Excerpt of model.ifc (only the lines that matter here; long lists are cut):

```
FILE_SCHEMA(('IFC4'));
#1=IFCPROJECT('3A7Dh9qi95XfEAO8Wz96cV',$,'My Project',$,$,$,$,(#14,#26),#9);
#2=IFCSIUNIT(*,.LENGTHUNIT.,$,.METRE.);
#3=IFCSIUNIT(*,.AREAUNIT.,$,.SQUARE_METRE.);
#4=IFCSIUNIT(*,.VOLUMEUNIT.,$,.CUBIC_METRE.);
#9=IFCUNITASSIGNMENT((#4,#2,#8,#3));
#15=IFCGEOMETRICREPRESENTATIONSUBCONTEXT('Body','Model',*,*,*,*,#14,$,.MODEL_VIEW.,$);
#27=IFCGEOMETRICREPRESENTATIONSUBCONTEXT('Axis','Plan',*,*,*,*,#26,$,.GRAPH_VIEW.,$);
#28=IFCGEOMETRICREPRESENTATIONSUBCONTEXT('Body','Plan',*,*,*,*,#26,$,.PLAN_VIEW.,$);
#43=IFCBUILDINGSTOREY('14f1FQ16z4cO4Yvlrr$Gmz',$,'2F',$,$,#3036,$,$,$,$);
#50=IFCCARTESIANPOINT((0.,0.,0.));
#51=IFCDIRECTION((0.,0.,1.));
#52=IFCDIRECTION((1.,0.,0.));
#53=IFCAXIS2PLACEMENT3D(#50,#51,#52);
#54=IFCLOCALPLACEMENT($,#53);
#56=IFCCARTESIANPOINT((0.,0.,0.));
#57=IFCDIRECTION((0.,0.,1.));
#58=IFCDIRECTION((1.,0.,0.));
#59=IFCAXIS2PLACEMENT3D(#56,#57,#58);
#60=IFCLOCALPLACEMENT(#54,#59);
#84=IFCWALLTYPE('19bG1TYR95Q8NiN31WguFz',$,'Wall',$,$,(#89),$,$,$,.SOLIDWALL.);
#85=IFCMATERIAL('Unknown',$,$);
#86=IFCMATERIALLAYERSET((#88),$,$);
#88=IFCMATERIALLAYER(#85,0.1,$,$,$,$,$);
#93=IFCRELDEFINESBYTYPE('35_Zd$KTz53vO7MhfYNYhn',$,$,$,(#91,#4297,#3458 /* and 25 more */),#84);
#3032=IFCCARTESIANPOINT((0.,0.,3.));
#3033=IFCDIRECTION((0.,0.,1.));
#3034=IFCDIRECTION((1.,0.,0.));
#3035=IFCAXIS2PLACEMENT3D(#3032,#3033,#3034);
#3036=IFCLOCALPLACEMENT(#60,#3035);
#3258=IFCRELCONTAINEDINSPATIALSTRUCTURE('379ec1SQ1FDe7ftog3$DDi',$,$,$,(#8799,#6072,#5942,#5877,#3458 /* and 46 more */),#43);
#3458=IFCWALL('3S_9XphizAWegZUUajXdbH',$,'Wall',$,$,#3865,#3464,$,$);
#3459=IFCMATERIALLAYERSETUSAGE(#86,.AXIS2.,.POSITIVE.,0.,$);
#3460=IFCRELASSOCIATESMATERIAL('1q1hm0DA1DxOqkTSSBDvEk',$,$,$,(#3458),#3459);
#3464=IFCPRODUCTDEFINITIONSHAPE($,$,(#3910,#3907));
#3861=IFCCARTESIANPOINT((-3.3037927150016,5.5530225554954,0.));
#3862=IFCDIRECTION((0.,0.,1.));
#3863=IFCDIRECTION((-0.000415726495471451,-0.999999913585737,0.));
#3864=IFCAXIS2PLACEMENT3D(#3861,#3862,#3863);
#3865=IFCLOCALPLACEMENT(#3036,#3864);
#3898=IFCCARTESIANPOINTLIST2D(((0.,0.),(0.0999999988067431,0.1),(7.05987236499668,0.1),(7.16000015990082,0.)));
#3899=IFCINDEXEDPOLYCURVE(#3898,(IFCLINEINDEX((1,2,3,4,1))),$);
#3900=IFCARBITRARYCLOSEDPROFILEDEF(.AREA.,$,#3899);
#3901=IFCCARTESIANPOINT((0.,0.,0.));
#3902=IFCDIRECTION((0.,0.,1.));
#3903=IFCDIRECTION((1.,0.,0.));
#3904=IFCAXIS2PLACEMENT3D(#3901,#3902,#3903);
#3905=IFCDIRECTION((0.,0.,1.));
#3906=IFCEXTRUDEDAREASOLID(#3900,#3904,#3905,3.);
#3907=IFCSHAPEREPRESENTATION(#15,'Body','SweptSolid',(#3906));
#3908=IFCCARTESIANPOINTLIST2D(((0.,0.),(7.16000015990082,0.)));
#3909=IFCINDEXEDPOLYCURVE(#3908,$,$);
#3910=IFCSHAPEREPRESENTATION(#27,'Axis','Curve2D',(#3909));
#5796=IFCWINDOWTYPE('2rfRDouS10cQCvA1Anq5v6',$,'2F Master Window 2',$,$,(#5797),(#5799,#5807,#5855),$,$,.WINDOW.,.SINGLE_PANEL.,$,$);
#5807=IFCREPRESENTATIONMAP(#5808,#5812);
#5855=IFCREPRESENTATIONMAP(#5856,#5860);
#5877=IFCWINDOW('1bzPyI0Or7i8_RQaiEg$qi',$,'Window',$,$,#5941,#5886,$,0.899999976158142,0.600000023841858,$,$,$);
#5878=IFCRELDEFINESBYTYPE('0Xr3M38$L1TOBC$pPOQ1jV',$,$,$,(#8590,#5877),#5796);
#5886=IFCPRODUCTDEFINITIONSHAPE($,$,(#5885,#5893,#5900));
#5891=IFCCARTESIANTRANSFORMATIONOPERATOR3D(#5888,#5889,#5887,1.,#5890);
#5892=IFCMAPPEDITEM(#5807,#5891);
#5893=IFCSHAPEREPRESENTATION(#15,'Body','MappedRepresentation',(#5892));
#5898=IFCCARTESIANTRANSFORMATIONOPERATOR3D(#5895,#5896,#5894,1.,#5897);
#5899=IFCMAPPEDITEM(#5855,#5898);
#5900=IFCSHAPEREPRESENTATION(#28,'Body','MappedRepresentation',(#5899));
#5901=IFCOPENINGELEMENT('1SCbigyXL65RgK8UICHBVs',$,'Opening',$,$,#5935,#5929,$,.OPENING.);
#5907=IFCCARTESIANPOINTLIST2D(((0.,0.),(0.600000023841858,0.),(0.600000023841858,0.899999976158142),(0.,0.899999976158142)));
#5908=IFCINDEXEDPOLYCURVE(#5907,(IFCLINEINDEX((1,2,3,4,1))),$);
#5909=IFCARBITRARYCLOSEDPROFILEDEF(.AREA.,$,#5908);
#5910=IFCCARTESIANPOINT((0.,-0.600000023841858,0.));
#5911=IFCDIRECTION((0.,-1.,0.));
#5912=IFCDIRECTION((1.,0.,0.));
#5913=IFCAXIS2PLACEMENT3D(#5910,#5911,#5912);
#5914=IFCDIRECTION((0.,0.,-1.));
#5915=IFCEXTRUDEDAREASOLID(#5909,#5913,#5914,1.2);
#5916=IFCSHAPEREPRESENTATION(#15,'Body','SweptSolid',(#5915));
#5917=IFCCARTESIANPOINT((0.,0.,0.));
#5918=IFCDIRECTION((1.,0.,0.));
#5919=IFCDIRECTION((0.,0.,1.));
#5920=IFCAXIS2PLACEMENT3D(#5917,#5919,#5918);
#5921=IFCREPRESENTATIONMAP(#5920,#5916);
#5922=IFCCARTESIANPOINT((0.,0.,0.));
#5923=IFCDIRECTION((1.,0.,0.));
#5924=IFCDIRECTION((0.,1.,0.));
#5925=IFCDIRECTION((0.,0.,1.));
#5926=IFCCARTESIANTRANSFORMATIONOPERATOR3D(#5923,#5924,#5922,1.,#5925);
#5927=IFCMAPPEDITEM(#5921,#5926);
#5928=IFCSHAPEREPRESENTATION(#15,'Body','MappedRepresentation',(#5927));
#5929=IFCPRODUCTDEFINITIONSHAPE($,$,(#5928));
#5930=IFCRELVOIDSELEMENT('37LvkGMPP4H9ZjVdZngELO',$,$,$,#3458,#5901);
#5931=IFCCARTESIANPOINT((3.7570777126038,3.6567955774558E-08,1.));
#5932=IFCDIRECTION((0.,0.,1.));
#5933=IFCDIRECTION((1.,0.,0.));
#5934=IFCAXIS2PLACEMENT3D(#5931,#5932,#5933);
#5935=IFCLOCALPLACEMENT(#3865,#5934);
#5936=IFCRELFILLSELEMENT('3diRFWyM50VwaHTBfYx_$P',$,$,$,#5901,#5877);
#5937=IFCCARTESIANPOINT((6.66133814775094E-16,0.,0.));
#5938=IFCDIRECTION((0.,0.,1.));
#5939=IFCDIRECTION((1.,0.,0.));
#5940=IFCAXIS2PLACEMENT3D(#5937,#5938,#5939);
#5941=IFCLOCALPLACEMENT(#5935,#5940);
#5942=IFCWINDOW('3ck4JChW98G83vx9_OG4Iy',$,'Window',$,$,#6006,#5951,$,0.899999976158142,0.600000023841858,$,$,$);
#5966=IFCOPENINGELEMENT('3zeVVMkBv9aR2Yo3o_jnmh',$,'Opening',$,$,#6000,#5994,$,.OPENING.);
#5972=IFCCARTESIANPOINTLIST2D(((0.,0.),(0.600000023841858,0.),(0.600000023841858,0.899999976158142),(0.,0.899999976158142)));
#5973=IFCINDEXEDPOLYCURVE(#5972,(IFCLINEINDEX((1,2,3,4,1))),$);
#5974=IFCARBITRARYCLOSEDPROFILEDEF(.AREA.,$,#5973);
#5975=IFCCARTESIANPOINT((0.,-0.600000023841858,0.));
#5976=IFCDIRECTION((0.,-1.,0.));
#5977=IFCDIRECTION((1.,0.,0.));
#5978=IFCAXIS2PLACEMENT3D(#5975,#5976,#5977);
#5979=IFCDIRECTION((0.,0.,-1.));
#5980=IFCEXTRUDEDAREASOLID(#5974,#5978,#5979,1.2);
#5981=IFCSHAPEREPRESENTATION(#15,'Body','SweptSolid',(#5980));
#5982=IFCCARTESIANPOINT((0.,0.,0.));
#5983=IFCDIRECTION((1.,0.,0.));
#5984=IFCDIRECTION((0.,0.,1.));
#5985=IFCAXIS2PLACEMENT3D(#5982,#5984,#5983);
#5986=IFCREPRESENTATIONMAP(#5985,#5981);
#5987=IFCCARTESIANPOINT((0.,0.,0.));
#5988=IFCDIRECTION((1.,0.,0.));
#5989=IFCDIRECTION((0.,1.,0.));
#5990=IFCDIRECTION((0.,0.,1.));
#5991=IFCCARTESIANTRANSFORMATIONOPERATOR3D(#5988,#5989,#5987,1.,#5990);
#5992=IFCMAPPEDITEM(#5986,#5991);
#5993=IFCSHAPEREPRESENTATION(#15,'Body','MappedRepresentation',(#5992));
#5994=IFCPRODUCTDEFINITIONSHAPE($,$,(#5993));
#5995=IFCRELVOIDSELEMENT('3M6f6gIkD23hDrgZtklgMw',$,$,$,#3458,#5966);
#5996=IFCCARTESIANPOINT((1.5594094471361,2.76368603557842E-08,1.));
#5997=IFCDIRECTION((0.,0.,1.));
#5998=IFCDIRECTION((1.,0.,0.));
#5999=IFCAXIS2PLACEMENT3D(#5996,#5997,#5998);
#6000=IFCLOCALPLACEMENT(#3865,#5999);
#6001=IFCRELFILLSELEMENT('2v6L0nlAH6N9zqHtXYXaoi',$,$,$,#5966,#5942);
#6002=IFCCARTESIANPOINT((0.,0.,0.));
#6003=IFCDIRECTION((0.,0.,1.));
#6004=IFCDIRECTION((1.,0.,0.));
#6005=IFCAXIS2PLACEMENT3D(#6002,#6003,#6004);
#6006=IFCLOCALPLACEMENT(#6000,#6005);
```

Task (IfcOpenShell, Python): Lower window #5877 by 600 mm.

```python
import numpy as np
import ifcopenshell
import ifcopenshell.api.geometry
import ifcopenshell.util.placement
import ifcopenshell.util.unit

model = ifcopenshell.open("model.ifc")
unit_scale = ifcopenshell.util.unit.calculate_unit_scale(model)

window = model.by_guid("1bzPyI0Or7i8_RQaiEg$qi")
opening = window.FillsVoids[0].RelatingOpeningElement
dz = -0.6 / unit_scale

shift = np.array([0.0, 0.0, dz])
# The window is placed relative to its opening, so it follows when the opening moves.
matrix = ifcopenshell.util.placement.get_local_placement(opening.ObjectPlacement)
matrix[:3, 3] += shift
ifcopenshell.api.geometry.edit_object_placement(
    model, product=opening, matrix=matrix, is_si=False, should_transform_children=True
)

print(f"moved by {dz * unit_scale:+.3f} m")

model.write("model_rev.ifc")
```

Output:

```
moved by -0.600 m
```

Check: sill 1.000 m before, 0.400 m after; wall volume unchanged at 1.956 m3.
